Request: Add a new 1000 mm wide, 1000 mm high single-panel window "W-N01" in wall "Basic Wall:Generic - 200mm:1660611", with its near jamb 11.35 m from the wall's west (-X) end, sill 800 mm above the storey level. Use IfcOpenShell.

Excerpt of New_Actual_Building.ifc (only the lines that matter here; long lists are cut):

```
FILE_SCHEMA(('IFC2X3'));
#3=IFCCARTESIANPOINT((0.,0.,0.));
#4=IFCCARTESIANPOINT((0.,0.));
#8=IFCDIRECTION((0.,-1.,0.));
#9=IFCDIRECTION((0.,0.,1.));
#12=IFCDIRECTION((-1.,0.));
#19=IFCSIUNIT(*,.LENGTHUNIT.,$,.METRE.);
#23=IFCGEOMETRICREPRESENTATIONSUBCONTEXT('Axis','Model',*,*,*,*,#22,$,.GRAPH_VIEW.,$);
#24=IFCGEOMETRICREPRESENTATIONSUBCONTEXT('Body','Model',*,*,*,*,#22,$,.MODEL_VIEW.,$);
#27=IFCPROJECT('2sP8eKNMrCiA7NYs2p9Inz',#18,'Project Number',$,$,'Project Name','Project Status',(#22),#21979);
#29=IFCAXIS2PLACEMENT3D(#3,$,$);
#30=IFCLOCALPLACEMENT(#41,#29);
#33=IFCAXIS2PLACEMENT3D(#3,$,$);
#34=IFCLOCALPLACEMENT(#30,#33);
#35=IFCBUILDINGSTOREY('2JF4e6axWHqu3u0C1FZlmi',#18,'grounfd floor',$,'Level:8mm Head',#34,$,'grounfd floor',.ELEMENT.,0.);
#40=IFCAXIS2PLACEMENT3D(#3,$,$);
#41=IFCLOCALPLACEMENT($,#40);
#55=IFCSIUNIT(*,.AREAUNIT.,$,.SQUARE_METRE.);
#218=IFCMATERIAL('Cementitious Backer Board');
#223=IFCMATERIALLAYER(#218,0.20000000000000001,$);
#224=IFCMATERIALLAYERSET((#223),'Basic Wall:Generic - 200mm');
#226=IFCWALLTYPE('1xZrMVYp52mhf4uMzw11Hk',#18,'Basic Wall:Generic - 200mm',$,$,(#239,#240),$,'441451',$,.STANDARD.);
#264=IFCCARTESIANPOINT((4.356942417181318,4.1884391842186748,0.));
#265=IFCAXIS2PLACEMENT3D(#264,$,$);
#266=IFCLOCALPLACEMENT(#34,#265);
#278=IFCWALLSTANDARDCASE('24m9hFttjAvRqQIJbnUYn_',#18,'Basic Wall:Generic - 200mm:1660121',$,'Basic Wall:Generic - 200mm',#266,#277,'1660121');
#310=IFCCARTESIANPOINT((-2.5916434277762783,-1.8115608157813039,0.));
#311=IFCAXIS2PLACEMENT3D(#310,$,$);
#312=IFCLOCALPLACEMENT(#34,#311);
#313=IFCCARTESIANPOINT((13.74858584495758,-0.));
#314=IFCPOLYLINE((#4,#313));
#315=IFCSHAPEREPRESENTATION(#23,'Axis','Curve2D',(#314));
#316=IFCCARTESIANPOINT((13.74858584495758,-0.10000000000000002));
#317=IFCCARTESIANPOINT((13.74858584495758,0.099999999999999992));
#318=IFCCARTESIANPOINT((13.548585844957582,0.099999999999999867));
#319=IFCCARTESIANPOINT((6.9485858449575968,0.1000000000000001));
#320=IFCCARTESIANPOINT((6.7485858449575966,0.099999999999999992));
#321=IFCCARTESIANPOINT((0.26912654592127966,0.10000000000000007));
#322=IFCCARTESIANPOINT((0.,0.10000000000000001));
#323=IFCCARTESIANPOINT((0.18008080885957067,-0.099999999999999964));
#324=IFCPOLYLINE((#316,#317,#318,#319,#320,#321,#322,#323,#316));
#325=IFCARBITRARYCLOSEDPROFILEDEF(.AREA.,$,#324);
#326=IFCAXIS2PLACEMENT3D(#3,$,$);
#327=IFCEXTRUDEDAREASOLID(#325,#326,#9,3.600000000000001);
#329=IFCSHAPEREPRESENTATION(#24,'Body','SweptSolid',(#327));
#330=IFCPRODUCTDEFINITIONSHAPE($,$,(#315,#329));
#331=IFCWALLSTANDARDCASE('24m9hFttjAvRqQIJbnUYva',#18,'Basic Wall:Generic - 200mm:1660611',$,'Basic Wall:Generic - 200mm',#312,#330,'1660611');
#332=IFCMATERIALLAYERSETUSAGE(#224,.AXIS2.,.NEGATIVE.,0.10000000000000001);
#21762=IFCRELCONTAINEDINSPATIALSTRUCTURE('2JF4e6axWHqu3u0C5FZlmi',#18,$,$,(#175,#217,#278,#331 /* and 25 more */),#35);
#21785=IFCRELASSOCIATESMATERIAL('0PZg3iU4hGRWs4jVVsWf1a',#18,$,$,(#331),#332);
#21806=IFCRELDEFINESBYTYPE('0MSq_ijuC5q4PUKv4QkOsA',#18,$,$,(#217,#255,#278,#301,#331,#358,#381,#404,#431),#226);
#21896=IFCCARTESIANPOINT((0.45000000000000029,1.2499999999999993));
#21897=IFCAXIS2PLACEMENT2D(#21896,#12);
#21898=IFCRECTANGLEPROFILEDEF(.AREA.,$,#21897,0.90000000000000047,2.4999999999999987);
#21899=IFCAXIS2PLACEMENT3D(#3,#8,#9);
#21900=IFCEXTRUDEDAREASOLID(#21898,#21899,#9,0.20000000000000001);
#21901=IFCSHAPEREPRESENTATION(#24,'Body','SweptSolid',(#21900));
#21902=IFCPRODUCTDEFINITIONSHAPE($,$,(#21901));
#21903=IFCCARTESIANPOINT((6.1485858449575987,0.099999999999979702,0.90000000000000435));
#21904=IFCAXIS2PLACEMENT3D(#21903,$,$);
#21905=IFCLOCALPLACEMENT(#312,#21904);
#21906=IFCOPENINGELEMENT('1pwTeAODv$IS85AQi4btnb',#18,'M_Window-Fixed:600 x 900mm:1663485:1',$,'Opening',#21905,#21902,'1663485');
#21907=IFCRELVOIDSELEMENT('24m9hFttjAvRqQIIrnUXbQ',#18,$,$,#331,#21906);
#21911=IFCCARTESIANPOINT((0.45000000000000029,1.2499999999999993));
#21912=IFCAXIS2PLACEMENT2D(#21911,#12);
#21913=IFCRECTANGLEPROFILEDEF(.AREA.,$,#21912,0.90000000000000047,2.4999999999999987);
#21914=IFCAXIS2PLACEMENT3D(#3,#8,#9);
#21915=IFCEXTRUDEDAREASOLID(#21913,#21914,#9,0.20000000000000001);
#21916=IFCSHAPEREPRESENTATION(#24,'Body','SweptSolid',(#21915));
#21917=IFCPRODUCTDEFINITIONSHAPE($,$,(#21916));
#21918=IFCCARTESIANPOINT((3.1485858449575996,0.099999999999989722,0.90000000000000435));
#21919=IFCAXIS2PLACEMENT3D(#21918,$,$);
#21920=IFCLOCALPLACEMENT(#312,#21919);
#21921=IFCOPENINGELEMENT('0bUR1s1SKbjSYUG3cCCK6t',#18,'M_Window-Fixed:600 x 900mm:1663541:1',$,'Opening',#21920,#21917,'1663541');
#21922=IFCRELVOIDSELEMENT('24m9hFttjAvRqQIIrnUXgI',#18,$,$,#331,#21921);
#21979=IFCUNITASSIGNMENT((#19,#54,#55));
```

```python
import numpy as np
import ifcopenshell
import ifcopenshell.api.feature
import ifcopenshell.api.geometry
import ifcopenshell.api.root
import ifcopenshell.api.spatial
import ifcopenshell.api.type
import ifcopenshell.geom
import ifcopenshell.util.element
import ifcopenshell.util.placement
import ifcopenshell.util.representation
import ifcopenshell.util.shape
import ifcopenshell.util.unit

model = ifcopenshell.open("New_Actual_Building.ifc")
unit_scale = ifcopenshell.util.unit.calculate_unit_scale(model)
settings = ifcopenshell.geom.settings()


def volume(element):
    """Net volume in cubic metres, openings subtracted."""
    shape = ifcopenshell.geom.create_shape(settings, element)
    return ifcopenshell.util.shape.get_volume(shape.geometry)


wall = model.by_id(331)
storey = ifcopenshell.util.element.get_container(wall, ifc_class="IfcBuildingStorey")
context = ifcopenshell.util.representation.get_context(model, "Model", "Body", "MODEL_VIEW")
before = volume(wall)

width, height, from_end, sill = 1, 1, 11.35, 0.8  # metres

# The wall runs along its own X axis, and the end named is its -X end.
wall_shape = ifcopenshell.geom.create_shape(settings, wall)
x, y, z = ifcopenshell.util.shape.get_vertices(wall_shape.geometry).T
start = x.min() + from_end
face, thickness = float(y.min()), float(y.max() - y.min())
wall_matrix = ifcopenshell.util.placement.get_local_placement(wall.ObjectPlacement)
level = ifcopenshell.util.placement.get_local_placement(storey.ObjectPlacement)[2, 3]


def in_wall(x, y):
    """Placement at x, y metres in the wall's axes, at sill height."""
    matrix = wall_matrix.copy()
    matrix[:, 3] = wall_matrix @ np.array([x / unit_scale, y / unit_scale, 0.0, 1.0])
    matrix[2, 3] = level + sill / unit_scale
    return matrix


# Opening: a box that overshoots both wall faces by 50 mm.
opening = ifcopenshell.api.root.create_entity(model, ifc_class="IfcOpeningElement")
box = ifcopenshell.api.geometry.add_wall_representation(
    model, context=context, length=width, height=height, thickness=thickness + 0.1
)
ifcopenshell.api.geometry.assign_representation(model, product=opening, representation=box)
ifcopenshell.api.geometry.edit_object_placement(model, product=opening, matrix=in_wall(start, face - 0.05), is_si=False)
ifcopenshell.api.feature.add_feature(model, feature=opening, element=wall)

window = ifcopenshell.api.root.create_entity(model, ifc_class="IfcWindow", name="W-N01")
window.OverallWidth, window.OverallHeight = width / unit_scale, height / unit_scale
body = ifcopenshell.api.geometry.add_window_representation(
    model,
    context=context,
    overall_width=window.OverallWidth,
    overall_height=window.OverallHeight,
    partition_type="SINGLE_PANEL",
)
ifcopenshell.api.geometry.assign_representation(model, product=window, representation=body)
ifcopenshell.api.spatial.assign_container(model, products=[window], relating_structure=storey)
fills = ifcopenshell.api.feature.add_filling(model, opening=opening, element=window)
fills.OwnerHistory = window.OwnerHistory  # required in IFC2X3

# IFC2X3 keeps the operation on the window style.
style = ifcopenshell.api.root.create_entity(model, ifc_class="IfcWindowStyle", name="W-N01")
style.OperationType, style.ConstructionType = "SINGLE_PANEL", "NOTDEFINED"
style.ParameterTakesPrecedence = style.Sizeable = False
ifcopenshell.api.type.assign_type(model, related_objects=[window], relating_type=style)

# Centre the window in the wall's thickness.
ifcopenshell.api.geometry.edit_object_placement(model, product=window, matrix=in_wall(start, face), is_si=False)
window_shape = ifcopenshell.geom.create_shape(settings, window)
depth = ifcopenshell.util.shape.get_vertices(window_shape.geometry)[:, 1]
offset = face + thickness / 2 - (depth.min() + depth.max()) / 2
ifcopenshell.api.geometry.edit_object_placement(model, product=window, matrix=in_wall(start, offset), is_si=False)

after = volume(wall)

print(f"wall volume {before:.3f} -> {after:.3f} m3")

model.write("New_Actual_Building-out.ifc")
```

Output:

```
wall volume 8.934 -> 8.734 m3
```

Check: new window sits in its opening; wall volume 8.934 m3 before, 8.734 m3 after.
